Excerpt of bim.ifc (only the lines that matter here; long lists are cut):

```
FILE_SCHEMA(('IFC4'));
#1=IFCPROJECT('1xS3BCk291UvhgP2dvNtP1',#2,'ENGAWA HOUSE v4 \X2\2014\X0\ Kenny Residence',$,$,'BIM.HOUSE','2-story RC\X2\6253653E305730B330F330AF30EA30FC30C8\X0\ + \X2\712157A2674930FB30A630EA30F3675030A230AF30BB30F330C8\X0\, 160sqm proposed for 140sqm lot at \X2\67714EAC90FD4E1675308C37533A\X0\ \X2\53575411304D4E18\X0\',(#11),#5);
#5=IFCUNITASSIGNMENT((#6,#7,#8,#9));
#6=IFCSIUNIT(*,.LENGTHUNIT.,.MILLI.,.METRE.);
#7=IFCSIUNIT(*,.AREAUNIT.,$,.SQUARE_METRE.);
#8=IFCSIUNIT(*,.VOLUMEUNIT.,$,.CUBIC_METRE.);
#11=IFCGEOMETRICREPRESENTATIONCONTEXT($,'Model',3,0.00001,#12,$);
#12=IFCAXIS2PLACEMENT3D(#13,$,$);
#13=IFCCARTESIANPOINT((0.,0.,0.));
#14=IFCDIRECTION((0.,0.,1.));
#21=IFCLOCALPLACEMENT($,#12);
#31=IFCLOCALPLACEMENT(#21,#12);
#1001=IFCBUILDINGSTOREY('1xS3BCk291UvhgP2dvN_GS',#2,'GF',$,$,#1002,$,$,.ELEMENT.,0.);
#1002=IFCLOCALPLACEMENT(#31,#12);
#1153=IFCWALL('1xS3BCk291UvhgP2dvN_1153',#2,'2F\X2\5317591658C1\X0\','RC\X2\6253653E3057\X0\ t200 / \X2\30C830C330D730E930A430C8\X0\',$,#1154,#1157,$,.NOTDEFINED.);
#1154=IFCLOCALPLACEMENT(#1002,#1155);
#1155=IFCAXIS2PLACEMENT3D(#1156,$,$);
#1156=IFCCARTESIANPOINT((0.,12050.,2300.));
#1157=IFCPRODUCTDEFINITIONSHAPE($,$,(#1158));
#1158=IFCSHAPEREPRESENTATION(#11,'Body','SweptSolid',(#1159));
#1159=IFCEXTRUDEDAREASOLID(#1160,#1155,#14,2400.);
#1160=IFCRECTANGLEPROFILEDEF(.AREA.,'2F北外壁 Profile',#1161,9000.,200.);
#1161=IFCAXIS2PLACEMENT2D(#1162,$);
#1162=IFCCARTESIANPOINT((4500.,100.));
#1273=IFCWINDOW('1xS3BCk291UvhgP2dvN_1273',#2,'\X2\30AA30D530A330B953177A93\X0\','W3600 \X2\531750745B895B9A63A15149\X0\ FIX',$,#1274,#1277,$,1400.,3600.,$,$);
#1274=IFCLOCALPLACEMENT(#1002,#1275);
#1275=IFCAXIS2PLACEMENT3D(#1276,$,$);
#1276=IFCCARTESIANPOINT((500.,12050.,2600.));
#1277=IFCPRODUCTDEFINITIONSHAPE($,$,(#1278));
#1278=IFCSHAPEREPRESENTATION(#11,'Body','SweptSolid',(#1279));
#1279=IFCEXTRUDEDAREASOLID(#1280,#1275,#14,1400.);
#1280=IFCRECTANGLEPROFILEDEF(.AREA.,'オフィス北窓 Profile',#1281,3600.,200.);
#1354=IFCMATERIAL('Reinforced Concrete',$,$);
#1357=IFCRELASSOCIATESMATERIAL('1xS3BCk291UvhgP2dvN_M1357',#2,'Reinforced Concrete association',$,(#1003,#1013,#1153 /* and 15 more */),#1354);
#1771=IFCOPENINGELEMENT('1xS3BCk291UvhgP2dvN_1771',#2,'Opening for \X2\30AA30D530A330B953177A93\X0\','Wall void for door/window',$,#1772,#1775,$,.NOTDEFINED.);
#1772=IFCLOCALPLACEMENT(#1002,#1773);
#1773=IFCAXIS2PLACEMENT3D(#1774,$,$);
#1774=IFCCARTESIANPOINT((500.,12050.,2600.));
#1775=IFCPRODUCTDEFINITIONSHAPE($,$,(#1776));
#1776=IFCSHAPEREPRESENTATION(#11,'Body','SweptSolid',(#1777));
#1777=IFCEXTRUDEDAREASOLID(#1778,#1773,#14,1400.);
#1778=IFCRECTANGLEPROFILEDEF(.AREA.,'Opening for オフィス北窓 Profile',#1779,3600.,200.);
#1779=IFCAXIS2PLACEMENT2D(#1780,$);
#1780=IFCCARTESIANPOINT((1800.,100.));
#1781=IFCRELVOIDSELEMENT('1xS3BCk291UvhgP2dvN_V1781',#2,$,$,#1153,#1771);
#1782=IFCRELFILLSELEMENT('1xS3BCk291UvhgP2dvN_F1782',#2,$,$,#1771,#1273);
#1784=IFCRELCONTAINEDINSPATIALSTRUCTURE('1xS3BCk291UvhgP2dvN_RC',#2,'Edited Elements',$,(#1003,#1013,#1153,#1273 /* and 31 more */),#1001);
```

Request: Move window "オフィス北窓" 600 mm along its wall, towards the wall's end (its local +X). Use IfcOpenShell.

```python
import ifcopenshell
import ifcopenshell.api.geometry
import ifcopenshell.util.placement
import ifcopenshell.util.unit

model = ifcopenshell.open("bim.ifc")
unit_scale = ifcopenshell.util.unit.calculate_unit_scale(model)

window = model.by_id(1273)
opening = window.FillsVoids[0].RelatingOpeningElement
wall = opening.VoidsElements[0].RelatingBuildingElement

wall_matrix = ifcopenshell.util.placement.get_local_placement(wall.ObjectPlacement)
shift = wall_matrix[:3, 0] * 0.6 / unit_scale
before = ifcopenshell.util.placement.get_local_placement(window.ObjectPlacement)[:3, 3].copy()

# The window is not placed relative to its opening, so move both.
for product in (opening, window):
    matrix = ifcopenshell.util.placement.get_local_placement(product.ObjectPlacement)
    matrix[:3, 3] += shift
    ifcopenshell.api.geometry.edit_object_placement(model, product=product, matrix=matrix, is_si=False)

after = ifcopenshell.util.placement.get_local_placement(window.ObjectPlacement)[:3, 3]
print("window moved by", (after - before).round(3) + 0.0)

model.write("bim_edited.ifc")
```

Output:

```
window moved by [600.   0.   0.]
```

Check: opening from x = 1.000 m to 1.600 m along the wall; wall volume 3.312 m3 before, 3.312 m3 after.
